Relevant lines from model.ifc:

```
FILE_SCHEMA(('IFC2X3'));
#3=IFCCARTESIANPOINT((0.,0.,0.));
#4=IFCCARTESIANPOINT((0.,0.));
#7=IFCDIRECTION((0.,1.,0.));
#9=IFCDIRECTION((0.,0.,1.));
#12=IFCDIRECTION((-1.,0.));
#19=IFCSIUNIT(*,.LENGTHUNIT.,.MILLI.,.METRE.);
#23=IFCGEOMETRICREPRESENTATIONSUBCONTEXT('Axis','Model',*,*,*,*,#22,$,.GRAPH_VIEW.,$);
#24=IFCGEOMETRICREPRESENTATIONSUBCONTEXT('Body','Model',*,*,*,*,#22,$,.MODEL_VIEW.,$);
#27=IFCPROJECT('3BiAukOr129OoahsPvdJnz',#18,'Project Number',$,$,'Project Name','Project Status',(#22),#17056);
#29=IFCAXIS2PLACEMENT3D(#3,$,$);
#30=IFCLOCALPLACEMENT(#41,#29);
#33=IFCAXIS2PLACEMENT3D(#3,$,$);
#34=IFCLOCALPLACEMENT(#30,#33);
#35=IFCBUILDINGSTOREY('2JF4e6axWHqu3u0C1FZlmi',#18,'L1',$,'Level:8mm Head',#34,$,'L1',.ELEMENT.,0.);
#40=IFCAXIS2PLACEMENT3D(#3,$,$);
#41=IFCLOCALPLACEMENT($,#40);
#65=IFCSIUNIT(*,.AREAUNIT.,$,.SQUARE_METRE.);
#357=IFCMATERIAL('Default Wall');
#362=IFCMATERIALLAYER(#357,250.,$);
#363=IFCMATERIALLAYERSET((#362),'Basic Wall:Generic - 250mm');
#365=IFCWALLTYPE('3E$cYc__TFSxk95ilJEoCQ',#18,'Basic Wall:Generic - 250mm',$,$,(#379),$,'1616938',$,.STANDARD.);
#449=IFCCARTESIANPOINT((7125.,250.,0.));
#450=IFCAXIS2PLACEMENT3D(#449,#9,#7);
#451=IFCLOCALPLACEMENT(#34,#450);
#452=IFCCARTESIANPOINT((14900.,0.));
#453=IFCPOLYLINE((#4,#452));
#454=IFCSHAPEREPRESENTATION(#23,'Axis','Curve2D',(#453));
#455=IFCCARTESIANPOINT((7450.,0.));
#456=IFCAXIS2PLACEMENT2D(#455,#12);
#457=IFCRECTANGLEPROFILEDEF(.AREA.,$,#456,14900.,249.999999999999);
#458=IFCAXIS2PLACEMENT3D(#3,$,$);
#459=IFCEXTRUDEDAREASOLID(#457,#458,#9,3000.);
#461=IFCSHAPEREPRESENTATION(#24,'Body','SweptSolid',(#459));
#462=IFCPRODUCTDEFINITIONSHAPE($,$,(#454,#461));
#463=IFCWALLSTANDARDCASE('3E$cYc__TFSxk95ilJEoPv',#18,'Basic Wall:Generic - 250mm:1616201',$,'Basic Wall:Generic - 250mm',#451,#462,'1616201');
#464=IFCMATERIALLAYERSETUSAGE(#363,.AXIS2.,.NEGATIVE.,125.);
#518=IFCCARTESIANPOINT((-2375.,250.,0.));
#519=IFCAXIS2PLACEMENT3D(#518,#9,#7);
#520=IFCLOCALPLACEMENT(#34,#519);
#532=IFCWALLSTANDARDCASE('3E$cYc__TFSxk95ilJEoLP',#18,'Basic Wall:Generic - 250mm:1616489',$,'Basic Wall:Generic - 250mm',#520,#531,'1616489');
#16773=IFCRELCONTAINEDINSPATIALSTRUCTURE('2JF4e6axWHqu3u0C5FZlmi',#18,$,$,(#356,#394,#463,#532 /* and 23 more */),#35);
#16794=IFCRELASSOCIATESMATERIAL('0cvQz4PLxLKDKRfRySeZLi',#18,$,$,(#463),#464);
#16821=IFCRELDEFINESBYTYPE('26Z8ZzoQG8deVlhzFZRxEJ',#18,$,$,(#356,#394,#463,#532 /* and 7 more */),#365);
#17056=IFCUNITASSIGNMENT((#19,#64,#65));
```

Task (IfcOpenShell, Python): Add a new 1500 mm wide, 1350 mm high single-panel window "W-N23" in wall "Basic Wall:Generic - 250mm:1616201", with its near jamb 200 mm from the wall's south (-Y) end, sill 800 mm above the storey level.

```python
import numpy as np
import ifcopenshell
import ifcopenshell.api.feature
import ifcopenshell.api.geometry
import ifcopenshell.api.root
import ifcopenshell.api.spatial
import ifcopenshell.api.type
import ifcopenshell.geom
import ifcopenshell.util.element
import ifcopenshell.util.placement
import ifcopenshell.util.representation
import ifcopenshell.util.shape
import ifcopenshell.util.unit

model = ifcopenshell.open("model.ifc")
unit_scale = ifcopenshell.util.unit.calculate_unit_scale(model)
settings = ifcopenshell.geom.settings()


def volume(element):
    """Net volume in cubic metres, openings subtracted."""
    shape = ifcopenshell.geom.create_shape(settings, element)
    return ifcopenshell.util.shape.get_volume(shape.geometry)


wall = model.by_guid("3E$cYc__TFSxk95ilJEoPv")
storey = ifcopenshell.util.element.get_container(wall, ifc_class="IfcBuildingStorey")
context = ifcopenshell.util.representation.get_context(model, "Model", "Body", "MODEL_VIEW")
before = volume(wall)

width, height, from_end, sill = 1.5, 1.35, 0.2, 0.8  # metres

# The wall runs along its own X axis, and the end named is its -X end.
wall_shape = ifcopenshell.geom.create_shape(settings, wall)
x, y, z = ifcopenshell.util.shape.get_vertices(wall_shape.geometry).T
start = x.min() + from_end
face, thickness = float(y.min()), float(y.max() - y.min())
wall_matrix = ifcopenshell.util.placement.get_local_placement(wall.ObjectPlacement)
level = ifcopenshell.util.placement.get_local_placement(storey.ObjectPlacement)[2, 3]


def in_wall(x, y):
    """Placement at x, y metres in the wall's axes, at sill height."""
    matrix = wall_matrix.copy()
    matrix[:, 3] = wall_matrix @ np.array([x / unit_scale, y / unit_scale, 0.0, 1.0])
    matrix[2, 3] = level + sill / unit_scale
    return matrix


# Opening: a box that overshoots both wall faces by 50 mm.
opening = ifcopenshell.api.root.create_entity(model, ifc_class="IfcOpeningElement")
box = ifcopenshell.api.geometry.add_wall_representation(
    model, context=context, length=width, height=height, thickness=thickness + 0.1
)
ifcopenshell.api.geometry.assign_representation(model, product=opening, representation=box)
ifcopenshell.api.geometry.edit_object_placement(model, product=opening, matrix=in_wall(start, face - 0.05), is_si=False)
ifcopenshell.api.feature.add_feature(model, feature=opening, element=wall)

window = ifcopenshell.api.root.create_entity(model, ifc_class="IfcWindow", name="W-N23")
window.OverallWidth, window.OverallHeight = width / unit_scale, height / unit_scale
body = ifcopenshell.api.geometry.add_window_representation(
    model,
    context=context,
    overall_width=window.OverallWidth,
    overall_height=window.OverallHeight,
    partition_type="SINGLE_PANEL",
)
ifcopenshell.api.geometry.assign_representation(model, product=window, representation=body)
ifcopenshell.api.spatial.assign_container(model, products=[window], relating_structure=storey)
fills = ifcopenshell.api.feature.add_filling(model, opening=opening, element=window)
fills.OwnerHistory = window.OwnerHistory  # required in IFC2X3

# IFC2X3 keeps the operation on the window style.
style = ifcopenshell.api.root.create_entity(model, ifc_class="IfcWindowStyle", name="W-N23")
style.OperationType, style.ConstructionType = "SINGLE_PANEL", "NOTDEFINED"
style.ParameterTakesPrecedence = style.Sizeable = False
ifcopenshell.api.type.assign_type(model, related_objects=[window], relating_type=style)

# Centre the window in the wall's thickness.
ifcopenshell.api.geometry.edit_object_placement(model, product=window, matrix=in_wall(start, face), is_si=False)
window_shape = ifcopenshell.geom.create_shape(settings, window)
depth = ifcopenshell.util.shape.get_vertices(window_shape.geometry)[:, 1]
offset = face + thickness / 2 - (depth.min() + depth.max()) / 2
ifcopenshell.api.geometry.edit_object_placement(model, product=window, matrix=in_wall(start, offset), is_si=False)

after = volume(wall)

print(f"wall volume {before:.3f} -> {after:.3f} m3")

model.write("model_v2.ifc")
```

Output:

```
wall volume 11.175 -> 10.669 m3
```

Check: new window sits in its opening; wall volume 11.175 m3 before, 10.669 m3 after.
